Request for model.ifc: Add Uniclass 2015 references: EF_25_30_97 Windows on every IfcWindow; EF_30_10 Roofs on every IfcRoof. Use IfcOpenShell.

First a look at what the model holds.

```python
import ifcopenshell

model = ifcopenshell.open("model.ifc")
print(model.schema)
print("classifications:", [c.Name for c in model.by_type("IfcClassification")])
for ifc_class in ("IfcDoor", "IfcRoof", "IfcStair", "IfcWall", "IfcWindow"):
    print(ifc_class, len(model.by_type(ifc_class)))
```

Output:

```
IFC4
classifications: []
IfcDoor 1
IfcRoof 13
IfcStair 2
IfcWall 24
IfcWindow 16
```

```python
import ifcopenshell
import ifcopenshell.api.classification

model = ifcopenshell.open("model.ifc")

system = ifcopenshell.api.classification.add_classification(model, classification="Uniclass 2015")

codes = {
    "IfcWindow": ("EF_25_30_97", "Windows"),
    "IfcRoof": ("EF_30_10", "Roofs"),
}
for ifc_class, (code, name) in codes.items():
    products = model.by_type(ifc_class)
    ifcopenshell.api.classification.add_reference(
        model, products=products, classification=system, identification=code, name=name
    )
    print(code, len(products))

model.write("model_updated.ifc")
```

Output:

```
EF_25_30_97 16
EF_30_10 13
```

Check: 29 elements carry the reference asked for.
